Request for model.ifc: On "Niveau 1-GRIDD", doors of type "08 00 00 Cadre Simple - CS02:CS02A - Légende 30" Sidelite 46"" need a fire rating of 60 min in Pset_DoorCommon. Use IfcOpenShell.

First a look at what the model holds.

```python
import ifcopenshell
import ifcopenshell.util.element

model = ifcopenshell.open("model.ifc")
print(model.schema)
storey = next(s for s in model.by_type("IfcBuildingStorey") if s.Name == "Niveau 1-GRIDD")
doors = [e for e in ifcopenshell.util.element.get_decomposition(storey) if e.is_a("IfcDoor")]
seen = {}
for e in doors:
    element_type = ifcopenshell.util.element.get_type(e)
    key = (element_type.Name if element_type != e and element_type else None, ifcopenshell.util.element.get_pset(e, "Pset_DoorCommon", "FireRating"))
    seen[key] = seen.get(key, 0) + 1
for (name, value), count in sorted(seen.items(), key=str):
    print(count, "x", name, "|", value)
```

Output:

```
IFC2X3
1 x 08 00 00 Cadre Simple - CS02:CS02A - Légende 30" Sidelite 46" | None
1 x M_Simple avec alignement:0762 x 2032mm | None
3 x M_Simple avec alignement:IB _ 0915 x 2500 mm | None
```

```python
import ifcopenshell
import ifcopenshell.api.pset
import ifcopenshell.util.element

model = ifcopenshell.open("model.ifc")

storey = next(s for s in model.by_type("IfcBuildingStorey") if s.Name == "Niveau 1-GRIDD")
doors = [e for e in ifcopenshell.util.element.get_decomposition(storey) if e.is_a("IfcDoor")]

count = 0
for e in doors:
    element_type = ifcopenshell.util.element.get_type(e)
    if element_type in (None, e) or element_type.Name != '08 00 00 Cadre Simple - CS02:CS02A - Légende 30" Sidelite 46"':
        continue
    # add_pset returns the element's existing set when there is one.
    pset = ifcopenshell.api.pset.add_pset(model, product=e, name="Pset_DoorCommon")
    ifcopenshell.api.pset.edit_pset(model, pset=pset, properties={"FireRating": "60 min"})
    count += 1

print(count, "doors updated")

model.write("model_v2.ifc")
```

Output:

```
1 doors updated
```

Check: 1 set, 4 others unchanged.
